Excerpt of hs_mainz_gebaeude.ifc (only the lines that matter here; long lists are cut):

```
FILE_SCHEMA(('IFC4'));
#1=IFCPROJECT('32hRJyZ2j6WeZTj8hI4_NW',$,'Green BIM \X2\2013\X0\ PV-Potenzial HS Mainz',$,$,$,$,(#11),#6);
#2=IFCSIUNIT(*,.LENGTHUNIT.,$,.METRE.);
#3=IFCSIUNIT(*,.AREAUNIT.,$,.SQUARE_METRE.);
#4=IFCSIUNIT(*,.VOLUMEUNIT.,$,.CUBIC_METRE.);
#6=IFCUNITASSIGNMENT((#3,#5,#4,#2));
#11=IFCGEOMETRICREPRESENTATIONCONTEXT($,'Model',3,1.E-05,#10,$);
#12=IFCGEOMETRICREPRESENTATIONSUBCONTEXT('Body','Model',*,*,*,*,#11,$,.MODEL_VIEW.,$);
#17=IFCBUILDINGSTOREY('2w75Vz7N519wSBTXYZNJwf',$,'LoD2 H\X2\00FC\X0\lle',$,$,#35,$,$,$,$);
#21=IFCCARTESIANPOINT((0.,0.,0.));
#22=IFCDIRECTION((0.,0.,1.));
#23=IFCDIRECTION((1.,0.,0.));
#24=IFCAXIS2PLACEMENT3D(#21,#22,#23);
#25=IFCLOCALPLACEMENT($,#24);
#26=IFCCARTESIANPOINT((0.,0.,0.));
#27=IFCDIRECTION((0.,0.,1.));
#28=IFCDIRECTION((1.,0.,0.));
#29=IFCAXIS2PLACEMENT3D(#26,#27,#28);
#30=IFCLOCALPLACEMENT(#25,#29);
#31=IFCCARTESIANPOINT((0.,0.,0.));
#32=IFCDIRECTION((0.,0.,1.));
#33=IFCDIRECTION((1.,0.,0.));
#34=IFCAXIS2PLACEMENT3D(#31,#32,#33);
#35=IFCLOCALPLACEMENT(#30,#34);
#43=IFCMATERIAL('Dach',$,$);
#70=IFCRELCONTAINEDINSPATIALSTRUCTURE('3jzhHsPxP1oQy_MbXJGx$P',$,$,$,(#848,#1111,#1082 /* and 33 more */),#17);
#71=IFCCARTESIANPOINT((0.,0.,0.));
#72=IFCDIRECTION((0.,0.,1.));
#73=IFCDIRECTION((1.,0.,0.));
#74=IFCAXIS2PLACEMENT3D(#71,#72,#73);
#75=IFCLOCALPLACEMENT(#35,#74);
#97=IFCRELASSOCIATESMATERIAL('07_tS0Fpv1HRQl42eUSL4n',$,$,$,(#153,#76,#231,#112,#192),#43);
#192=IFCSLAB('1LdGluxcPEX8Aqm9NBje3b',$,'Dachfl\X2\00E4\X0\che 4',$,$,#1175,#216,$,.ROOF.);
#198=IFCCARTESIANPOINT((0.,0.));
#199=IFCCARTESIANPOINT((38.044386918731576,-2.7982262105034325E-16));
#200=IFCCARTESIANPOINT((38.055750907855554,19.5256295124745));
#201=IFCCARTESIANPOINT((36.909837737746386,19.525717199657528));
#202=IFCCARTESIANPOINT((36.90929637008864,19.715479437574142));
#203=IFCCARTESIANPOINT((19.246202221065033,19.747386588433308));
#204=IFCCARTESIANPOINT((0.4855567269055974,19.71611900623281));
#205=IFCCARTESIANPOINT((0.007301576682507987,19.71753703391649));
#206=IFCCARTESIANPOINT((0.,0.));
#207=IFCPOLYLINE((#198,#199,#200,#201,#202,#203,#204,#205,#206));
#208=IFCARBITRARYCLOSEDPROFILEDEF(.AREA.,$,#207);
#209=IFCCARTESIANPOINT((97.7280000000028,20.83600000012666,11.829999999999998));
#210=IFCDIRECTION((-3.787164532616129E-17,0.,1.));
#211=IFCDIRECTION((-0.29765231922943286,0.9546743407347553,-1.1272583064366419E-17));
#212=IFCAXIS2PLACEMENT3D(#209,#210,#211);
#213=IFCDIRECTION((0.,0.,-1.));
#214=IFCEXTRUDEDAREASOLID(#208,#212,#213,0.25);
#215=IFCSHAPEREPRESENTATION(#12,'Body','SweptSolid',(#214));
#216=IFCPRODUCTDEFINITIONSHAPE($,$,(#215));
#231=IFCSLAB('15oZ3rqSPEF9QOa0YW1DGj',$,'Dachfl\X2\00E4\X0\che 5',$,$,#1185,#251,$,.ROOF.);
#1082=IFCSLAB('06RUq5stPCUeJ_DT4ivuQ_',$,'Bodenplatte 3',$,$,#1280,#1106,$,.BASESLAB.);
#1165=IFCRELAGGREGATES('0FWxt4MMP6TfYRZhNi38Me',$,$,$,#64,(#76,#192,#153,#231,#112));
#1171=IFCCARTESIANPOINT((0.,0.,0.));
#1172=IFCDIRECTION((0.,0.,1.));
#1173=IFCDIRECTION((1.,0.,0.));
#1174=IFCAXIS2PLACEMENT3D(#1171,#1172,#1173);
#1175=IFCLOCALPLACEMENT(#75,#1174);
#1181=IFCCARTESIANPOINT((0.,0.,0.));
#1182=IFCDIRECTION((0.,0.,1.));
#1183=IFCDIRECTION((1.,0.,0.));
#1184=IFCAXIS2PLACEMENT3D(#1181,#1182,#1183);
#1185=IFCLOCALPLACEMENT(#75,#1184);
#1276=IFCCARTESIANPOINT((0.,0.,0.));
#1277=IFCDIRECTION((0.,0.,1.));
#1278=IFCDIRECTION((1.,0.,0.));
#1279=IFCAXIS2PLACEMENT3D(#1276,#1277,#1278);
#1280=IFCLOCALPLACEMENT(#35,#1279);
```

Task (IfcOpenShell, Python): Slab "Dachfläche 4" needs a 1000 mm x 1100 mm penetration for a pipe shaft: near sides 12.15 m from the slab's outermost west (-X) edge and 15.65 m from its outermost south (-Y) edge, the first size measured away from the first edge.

```python
import numpy as np
import ifcopenshell
import ifcopenshell.api.feature
import ifcopenshell.api.geometry
import ifcopenshell.api.root
import ifcopenshell.geom
import ifcopenshell.util.placement
import ifcopenshell.util.representation
import ifcopenshell.util.shape
import ifcopenshell.util.unit

model = ifcopenshell.open("hs_mainz_gebaeude.ifc")
unit_scale = ifcopenshell.util.unit.calculate_unit_scale(model)
settings = ifcopenshell.geom.settings()


def volume(element):
    """Net volume in cubic metres, openings subtracted."""
    shape = ifcopenshell.geom.create_shape(settings, element)
    return ifcopenshell.util.shape.get_volume(shape.geometry)


slab = model.by_guid("1LdGluxcPEX8Aqm9NBje3b")
before = volume(slab)

# Extent in the slab's own axes, in metres. The edges named are its -X and -Y sides.
slab_shape = ifcopenshell.geom.create_shape(settings, slab)
vertices = ifcopenshell.util.shape.get_vertices(slab_shape.geometry)
x_min, y_min, bottom = vertices.min(axis=0)
top = vertices[:, 2].max()

opening = ifcopenshell.api.root.create_entity(model, ifc_class="IfcOpeningElement", name="Pipe shaft opening", predefined_type="OPENING")
context = ifcopenshell.util.representation.get_context(model, "Model", "Body", "MODEL_VIEW")
width, depth = 1, 1.1
outline = [(0.0, 0.0), (width, 0.0), (width, depth), (0.0, depth), (0.0, 0.0)]
# Overshoot both faces by 50 mm so the cut is clean.
shape = ifcopenshell.api.geometry.add_slab_representation(
    model, context=context, depth=top - bottom + 0.1, polyline=outline
)
ifcopenshell.api.geometry.assign_representation(model, product=opening, representation=shape)

matrix = ifcopenshell.util.placement.get_local_placement(slab.ObjectPlacement)
matrix[:, 3] = matrix @ np.append(np.array([x_min + 12.15, y_min + 15.65, bottom - 0.05]) / unit_scale, 1.0)
ifcopenshell.api.geometry.edit_object_placement(model, product=opening, matrix=matrix, is_si=False)
ifcopenshell.api.feature.add_feature(model, feature=opening, element=slab)

after = volume(slab)

print(f"slab volume {before:.3f} -> {after:.3f} m3")

model.write("hs_mainz_gebaeude_v2.ifc")
```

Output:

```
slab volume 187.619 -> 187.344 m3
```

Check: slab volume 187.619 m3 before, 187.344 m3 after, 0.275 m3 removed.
